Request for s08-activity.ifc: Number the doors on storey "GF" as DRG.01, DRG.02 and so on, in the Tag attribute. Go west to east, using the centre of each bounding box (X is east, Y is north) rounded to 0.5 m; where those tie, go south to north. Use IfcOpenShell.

First a look at what the model holds.

```python
import ifcopenshell
import ifcopenshell.util.element
import ifcopenshell.util.placement

model = ifcopenshell.open("s08-activity.ifc")
print(model.schema)
storey = next(s for s in model.by_type("IfcBuildingStorey") if s.Name == "GF")
doors = [e for e in ifcopenshell.util.element.get_decomposition(storey) if e.is_a("IfcDoor")]
for e in sorted(doors, key=lambda e: e.id()):
    origin = ifcopenshell.util.placement.get_local_placement(e.ObjectPlacement)[:3, 3]
    print(e.id(), e.Tag, e.Name, origin.round(2) + 0.0, sep=" | ")
```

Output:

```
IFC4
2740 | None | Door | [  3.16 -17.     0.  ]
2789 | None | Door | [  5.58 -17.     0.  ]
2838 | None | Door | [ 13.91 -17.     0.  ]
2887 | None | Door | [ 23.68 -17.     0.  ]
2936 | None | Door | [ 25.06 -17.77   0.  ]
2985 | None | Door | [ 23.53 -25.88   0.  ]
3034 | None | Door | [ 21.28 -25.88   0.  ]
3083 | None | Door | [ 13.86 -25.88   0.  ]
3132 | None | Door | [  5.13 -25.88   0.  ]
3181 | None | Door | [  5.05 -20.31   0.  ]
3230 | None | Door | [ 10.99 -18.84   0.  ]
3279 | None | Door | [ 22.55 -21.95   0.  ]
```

```python
import ifcopenshell
import ifcopenshell.geom
import ifcopenshell.util.element
import ifcopenshell.util.shape

model = ifcopenshell.open("s08-activity.ifc")
settings = ifcopenshell.geom.settings()
settings.set("use-world-coords", True)


def centre(element):
    shape = ifcopenshell.geom.create_shape(settings, element)
    return ifcopenshell.util.shape.get_bbox_centroid(shape.geometry)


storey = next(s for s in model.by_type("IfcBuildingStorey") if s.Name == "GF")
doors = [e for e in ifcopenshell.util.element.get_decomposition(storey) if e.is_a("IfcDoor")]

# Insertion points can sit at a corner or the storey origin, so sort by the geometry (in metres).
centres = {e: centre(e) for e in doors}
doors.sort(key=lambda e: (round(centres[e][0] / 0.5), centres[e][1]))

for i, e in enumerate(doors, start=1):
    number = f"DRG.{i:02d}"
    e.Tag = number
    print(e.id(), number)

model.write("s08-activity_updated.ifc")
```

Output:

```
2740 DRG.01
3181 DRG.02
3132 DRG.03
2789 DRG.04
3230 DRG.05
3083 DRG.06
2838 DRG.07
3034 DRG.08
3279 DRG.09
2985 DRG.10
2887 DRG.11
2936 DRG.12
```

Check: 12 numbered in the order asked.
